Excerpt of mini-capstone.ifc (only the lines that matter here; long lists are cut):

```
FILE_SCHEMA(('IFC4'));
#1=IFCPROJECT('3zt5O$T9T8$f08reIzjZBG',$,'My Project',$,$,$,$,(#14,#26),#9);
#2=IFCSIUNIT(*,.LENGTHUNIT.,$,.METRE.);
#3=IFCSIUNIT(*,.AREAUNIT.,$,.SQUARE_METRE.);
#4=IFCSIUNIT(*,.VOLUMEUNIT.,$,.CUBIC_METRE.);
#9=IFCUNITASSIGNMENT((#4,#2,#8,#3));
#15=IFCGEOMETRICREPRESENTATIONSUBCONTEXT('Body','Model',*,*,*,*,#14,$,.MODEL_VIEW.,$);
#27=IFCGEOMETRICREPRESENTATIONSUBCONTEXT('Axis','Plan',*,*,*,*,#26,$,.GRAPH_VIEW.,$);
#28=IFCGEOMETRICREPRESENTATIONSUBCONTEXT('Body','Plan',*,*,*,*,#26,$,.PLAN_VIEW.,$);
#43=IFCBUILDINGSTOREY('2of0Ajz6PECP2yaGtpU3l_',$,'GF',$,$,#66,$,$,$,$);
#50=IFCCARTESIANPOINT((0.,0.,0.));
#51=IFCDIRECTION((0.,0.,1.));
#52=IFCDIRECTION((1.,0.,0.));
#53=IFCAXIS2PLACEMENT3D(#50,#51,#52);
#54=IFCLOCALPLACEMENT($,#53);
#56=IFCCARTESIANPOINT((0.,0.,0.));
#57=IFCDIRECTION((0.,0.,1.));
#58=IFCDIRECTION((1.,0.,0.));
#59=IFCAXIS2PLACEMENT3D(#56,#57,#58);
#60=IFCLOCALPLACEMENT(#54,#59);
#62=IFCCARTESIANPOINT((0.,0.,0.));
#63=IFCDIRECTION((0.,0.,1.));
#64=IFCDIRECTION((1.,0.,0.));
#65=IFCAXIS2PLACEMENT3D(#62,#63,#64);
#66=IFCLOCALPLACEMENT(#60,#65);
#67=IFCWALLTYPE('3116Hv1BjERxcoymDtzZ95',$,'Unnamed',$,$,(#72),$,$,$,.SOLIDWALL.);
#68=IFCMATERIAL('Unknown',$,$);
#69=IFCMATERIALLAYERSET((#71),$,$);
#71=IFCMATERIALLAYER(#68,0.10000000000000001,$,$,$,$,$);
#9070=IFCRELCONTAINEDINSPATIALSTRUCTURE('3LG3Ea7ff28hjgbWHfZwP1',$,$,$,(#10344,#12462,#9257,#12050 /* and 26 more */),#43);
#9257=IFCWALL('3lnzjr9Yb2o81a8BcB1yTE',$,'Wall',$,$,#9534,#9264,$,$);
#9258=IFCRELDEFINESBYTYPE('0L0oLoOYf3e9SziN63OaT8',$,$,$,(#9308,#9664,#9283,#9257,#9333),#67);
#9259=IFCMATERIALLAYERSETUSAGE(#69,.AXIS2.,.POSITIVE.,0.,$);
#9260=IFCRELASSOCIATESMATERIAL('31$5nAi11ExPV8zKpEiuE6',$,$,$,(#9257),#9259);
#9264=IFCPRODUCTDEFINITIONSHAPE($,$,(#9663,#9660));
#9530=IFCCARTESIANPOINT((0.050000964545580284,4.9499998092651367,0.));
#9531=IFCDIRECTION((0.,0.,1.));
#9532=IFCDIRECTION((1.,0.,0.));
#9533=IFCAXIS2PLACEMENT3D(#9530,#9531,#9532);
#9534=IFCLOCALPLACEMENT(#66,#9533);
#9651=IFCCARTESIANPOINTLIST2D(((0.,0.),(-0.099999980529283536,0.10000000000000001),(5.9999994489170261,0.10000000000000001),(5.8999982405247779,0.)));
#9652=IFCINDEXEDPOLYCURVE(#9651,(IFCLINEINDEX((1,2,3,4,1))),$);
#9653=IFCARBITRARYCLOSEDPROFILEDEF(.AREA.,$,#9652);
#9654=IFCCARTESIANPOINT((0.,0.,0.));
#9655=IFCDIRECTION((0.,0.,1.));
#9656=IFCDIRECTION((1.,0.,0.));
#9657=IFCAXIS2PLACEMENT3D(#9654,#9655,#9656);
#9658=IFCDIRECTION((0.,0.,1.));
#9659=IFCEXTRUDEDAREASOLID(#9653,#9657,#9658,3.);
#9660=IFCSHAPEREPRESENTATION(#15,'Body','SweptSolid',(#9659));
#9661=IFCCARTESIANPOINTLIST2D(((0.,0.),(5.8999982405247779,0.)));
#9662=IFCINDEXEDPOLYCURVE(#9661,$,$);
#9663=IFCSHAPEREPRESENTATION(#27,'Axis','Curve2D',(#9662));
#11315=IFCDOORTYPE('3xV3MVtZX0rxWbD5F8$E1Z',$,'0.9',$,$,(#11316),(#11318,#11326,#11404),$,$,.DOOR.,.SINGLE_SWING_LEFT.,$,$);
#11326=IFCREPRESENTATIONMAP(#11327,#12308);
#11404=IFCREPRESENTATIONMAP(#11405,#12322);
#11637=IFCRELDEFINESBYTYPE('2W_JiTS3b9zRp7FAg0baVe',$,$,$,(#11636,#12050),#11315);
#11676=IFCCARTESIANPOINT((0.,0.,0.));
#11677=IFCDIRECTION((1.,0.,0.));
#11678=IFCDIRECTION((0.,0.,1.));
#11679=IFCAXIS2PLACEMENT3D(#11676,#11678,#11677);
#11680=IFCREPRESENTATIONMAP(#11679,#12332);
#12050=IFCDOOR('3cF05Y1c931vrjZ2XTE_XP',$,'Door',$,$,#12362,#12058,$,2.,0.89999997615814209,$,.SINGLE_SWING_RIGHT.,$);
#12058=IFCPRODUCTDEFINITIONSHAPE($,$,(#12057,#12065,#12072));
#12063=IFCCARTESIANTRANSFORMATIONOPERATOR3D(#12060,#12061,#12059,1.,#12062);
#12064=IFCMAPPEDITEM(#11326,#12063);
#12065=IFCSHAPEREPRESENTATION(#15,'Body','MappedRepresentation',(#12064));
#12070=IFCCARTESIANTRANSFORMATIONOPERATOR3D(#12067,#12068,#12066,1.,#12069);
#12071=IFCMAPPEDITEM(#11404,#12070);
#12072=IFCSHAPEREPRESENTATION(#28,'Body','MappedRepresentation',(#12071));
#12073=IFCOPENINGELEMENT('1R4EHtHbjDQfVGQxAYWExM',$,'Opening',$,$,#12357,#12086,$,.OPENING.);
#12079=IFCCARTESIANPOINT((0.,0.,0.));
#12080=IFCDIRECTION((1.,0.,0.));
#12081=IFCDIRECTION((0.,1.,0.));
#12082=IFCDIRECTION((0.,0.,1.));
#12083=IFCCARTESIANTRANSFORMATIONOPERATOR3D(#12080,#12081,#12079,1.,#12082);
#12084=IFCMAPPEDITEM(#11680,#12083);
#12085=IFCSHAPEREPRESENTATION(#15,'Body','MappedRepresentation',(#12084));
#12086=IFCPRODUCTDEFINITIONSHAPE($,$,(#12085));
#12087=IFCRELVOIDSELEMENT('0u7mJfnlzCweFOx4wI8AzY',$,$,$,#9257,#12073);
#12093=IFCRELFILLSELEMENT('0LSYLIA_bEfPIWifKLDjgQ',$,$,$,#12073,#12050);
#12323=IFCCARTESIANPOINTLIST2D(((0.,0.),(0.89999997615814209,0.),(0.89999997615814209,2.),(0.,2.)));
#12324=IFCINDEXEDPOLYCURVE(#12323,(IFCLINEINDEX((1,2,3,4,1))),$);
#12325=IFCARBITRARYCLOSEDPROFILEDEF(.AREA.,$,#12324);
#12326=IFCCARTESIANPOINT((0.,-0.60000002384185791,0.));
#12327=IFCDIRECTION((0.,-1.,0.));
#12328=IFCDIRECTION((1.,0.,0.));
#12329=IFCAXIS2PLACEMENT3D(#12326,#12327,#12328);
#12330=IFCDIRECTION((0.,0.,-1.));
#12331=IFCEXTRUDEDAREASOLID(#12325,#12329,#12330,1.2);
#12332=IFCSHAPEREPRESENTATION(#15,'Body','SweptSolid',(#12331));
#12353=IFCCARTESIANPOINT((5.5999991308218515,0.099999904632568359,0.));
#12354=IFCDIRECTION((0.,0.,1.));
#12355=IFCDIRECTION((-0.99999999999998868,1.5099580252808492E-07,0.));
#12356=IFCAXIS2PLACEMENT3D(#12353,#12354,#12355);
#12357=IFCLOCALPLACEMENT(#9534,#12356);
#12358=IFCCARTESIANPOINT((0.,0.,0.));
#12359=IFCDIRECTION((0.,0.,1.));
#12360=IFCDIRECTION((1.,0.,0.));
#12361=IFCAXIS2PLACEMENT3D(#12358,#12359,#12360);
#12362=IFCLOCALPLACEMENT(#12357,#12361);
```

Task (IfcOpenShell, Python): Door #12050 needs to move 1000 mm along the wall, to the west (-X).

```python
import ifcopenshell
import ifcopenshell.api.geometry
import ifcopenshell.util.placement
import ifcopenshell.util.unit

model = ifcopenshell.open("mini-capstone.ifc")
unit_scale = ifcopenshell.util.unit.calculate_unit_scale(model)

door = model.by_guid("3cF05Y1c931vrjZ2XTE_XP")
opening = door.FillsVoids[0].RelatingOpeningElement
wall = opening.VoidsElements[0].RelatingBuildingElement

wall_matrix = ifcopenshell.util.placement.get_local_placement(wall.ObjectPlacement)
shift = wall_matrix[:3, 0] * -1 / unit_scale
before = ifcopenshell.util.placement.get_local_placement(door.ObjectPlacement)[:3, 3].copy()

# The door is placed relative to its opening, so it follows when the opening moves.
matrix = ifcopenshell.util.placement.get_local_placement(opening.ObjectPlacement)
matrix[:3, 3] += shift
ifcopenshell.api.geometry.edit_object_placement(
    model, product=opening, matrix=matrix, is_si=False, should_transform_children=True
)

after = ifcopenshell.util.placement.get_local_placement(door.ObjectPlacement)[:3, 3]
print("door moved by", (after - before).round(3) + 0.0)

model.write("mini-capstone_v2.ifc")
```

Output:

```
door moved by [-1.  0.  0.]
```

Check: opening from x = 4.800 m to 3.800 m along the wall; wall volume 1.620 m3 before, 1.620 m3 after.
